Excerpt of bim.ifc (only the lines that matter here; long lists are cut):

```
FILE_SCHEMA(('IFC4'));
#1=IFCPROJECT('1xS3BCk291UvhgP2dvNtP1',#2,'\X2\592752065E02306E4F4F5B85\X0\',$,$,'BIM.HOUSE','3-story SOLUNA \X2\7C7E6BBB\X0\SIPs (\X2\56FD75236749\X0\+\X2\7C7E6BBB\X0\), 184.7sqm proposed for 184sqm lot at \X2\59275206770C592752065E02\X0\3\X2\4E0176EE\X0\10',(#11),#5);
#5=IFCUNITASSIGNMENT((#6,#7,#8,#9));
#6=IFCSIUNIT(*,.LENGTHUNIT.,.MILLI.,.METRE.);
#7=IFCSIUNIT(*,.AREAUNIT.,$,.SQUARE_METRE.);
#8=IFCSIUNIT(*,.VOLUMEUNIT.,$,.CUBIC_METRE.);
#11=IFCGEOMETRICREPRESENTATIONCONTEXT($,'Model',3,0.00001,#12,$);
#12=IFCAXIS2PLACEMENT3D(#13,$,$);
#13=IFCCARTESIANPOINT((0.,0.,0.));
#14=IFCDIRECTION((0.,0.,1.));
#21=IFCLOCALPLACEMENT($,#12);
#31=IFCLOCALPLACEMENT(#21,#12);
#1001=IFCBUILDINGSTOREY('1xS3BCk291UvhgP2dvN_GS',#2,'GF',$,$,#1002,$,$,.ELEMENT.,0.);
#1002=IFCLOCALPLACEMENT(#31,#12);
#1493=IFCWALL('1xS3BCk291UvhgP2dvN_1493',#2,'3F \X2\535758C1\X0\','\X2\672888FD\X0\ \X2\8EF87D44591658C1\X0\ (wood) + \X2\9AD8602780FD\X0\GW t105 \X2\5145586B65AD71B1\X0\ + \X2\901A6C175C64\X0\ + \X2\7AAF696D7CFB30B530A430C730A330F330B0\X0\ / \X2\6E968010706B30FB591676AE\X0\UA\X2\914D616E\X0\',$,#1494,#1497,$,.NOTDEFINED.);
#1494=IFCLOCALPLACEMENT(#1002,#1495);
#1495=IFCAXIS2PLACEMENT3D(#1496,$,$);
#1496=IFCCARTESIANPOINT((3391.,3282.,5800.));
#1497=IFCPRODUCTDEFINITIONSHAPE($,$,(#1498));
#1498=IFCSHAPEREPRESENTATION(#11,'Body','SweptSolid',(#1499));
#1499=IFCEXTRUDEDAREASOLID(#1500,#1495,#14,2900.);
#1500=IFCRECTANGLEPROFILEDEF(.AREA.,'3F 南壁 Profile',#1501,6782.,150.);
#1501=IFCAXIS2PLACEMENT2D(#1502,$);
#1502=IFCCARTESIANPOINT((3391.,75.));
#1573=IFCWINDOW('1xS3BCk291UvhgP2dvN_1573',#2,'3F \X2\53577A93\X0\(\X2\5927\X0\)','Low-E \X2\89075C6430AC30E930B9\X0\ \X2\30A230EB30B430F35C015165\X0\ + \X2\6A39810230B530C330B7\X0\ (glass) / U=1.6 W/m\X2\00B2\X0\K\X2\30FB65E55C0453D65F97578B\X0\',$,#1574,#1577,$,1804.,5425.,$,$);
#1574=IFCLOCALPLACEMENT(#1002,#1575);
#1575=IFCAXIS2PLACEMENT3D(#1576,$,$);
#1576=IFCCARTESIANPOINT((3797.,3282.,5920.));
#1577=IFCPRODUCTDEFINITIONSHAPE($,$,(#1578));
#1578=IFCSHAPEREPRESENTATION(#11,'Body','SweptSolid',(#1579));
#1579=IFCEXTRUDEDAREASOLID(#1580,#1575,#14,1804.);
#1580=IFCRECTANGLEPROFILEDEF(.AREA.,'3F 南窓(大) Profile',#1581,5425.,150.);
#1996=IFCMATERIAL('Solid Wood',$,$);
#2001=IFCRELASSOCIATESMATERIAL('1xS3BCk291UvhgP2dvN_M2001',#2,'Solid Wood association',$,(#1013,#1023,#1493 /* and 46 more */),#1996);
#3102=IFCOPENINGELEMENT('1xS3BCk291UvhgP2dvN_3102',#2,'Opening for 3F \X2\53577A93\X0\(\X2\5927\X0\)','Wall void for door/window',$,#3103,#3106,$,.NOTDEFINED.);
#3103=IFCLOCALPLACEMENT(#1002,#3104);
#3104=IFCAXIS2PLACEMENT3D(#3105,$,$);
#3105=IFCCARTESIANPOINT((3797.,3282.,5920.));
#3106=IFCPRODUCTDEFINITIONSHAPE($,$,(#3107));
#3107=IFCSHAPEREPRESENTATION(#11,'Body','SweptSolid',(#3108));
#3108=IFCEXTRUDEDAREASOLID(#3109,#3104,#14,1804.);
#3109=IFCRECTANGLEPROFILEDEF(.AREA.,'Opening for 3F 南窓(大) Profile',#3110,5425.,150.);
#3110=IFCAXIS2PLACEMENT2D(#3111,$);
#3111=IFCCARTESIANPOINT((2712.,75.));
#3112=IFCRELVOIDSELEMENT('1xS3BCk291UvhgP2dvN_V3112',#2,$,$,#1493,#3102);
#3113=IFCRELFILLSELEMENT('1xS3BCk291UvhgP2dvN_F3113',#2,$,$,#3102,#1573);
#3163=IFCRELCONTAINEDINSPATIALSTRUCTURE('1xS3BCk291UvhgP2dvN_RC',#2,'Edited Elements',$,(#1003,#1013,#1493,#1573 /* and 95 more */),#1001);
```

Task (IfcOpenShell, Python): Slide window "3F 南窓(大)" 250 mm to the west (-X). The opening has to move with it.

```python
import ifcopenshell
import ifcopenshell.api.geometry
import ifcopenshell.util.placement

model = ifcopenshell.open("bim.ifc")

window = model.by_guid("1xS3BCk291UvhgP2dvN_1573")
opening = window.FillsVoids[0].RelatingOpeningElement
wall = opening.VoidsElements[0].RelatingBuildingElement

wall_matrix = ifcopenshell.util.placement.get_local_placement(wall.ObjectPlacement)
shift = wall_matrix[:3, 0] * -250.0
before = ifcopenshell.util.placement.get_local_placement(window.ObjectPlacement)[:3, 3].copy()

# The window is not placed relative to its opening, so move both.
for product in (opening, window):
    matrix = ifcopenshell.util.placement.get_local_placement(product.ObjectPlacement)
    matrix[:3, 3] += shift
    ifcopenshell.api.geometry.edit_object_placement(model, product=product, matrix=matrix, is_si=False)

after = ifcopenshell.util.placement.get_local_placement(window.ObjectPlacement)[:3, 3]
print("window moved by", (after - before).round(3) + 0.0)

model.write("bim_edited.ifc")
```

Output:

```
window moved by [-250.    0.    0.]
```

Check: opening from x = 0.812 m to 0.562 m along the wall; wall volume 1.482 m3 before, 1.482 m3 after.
